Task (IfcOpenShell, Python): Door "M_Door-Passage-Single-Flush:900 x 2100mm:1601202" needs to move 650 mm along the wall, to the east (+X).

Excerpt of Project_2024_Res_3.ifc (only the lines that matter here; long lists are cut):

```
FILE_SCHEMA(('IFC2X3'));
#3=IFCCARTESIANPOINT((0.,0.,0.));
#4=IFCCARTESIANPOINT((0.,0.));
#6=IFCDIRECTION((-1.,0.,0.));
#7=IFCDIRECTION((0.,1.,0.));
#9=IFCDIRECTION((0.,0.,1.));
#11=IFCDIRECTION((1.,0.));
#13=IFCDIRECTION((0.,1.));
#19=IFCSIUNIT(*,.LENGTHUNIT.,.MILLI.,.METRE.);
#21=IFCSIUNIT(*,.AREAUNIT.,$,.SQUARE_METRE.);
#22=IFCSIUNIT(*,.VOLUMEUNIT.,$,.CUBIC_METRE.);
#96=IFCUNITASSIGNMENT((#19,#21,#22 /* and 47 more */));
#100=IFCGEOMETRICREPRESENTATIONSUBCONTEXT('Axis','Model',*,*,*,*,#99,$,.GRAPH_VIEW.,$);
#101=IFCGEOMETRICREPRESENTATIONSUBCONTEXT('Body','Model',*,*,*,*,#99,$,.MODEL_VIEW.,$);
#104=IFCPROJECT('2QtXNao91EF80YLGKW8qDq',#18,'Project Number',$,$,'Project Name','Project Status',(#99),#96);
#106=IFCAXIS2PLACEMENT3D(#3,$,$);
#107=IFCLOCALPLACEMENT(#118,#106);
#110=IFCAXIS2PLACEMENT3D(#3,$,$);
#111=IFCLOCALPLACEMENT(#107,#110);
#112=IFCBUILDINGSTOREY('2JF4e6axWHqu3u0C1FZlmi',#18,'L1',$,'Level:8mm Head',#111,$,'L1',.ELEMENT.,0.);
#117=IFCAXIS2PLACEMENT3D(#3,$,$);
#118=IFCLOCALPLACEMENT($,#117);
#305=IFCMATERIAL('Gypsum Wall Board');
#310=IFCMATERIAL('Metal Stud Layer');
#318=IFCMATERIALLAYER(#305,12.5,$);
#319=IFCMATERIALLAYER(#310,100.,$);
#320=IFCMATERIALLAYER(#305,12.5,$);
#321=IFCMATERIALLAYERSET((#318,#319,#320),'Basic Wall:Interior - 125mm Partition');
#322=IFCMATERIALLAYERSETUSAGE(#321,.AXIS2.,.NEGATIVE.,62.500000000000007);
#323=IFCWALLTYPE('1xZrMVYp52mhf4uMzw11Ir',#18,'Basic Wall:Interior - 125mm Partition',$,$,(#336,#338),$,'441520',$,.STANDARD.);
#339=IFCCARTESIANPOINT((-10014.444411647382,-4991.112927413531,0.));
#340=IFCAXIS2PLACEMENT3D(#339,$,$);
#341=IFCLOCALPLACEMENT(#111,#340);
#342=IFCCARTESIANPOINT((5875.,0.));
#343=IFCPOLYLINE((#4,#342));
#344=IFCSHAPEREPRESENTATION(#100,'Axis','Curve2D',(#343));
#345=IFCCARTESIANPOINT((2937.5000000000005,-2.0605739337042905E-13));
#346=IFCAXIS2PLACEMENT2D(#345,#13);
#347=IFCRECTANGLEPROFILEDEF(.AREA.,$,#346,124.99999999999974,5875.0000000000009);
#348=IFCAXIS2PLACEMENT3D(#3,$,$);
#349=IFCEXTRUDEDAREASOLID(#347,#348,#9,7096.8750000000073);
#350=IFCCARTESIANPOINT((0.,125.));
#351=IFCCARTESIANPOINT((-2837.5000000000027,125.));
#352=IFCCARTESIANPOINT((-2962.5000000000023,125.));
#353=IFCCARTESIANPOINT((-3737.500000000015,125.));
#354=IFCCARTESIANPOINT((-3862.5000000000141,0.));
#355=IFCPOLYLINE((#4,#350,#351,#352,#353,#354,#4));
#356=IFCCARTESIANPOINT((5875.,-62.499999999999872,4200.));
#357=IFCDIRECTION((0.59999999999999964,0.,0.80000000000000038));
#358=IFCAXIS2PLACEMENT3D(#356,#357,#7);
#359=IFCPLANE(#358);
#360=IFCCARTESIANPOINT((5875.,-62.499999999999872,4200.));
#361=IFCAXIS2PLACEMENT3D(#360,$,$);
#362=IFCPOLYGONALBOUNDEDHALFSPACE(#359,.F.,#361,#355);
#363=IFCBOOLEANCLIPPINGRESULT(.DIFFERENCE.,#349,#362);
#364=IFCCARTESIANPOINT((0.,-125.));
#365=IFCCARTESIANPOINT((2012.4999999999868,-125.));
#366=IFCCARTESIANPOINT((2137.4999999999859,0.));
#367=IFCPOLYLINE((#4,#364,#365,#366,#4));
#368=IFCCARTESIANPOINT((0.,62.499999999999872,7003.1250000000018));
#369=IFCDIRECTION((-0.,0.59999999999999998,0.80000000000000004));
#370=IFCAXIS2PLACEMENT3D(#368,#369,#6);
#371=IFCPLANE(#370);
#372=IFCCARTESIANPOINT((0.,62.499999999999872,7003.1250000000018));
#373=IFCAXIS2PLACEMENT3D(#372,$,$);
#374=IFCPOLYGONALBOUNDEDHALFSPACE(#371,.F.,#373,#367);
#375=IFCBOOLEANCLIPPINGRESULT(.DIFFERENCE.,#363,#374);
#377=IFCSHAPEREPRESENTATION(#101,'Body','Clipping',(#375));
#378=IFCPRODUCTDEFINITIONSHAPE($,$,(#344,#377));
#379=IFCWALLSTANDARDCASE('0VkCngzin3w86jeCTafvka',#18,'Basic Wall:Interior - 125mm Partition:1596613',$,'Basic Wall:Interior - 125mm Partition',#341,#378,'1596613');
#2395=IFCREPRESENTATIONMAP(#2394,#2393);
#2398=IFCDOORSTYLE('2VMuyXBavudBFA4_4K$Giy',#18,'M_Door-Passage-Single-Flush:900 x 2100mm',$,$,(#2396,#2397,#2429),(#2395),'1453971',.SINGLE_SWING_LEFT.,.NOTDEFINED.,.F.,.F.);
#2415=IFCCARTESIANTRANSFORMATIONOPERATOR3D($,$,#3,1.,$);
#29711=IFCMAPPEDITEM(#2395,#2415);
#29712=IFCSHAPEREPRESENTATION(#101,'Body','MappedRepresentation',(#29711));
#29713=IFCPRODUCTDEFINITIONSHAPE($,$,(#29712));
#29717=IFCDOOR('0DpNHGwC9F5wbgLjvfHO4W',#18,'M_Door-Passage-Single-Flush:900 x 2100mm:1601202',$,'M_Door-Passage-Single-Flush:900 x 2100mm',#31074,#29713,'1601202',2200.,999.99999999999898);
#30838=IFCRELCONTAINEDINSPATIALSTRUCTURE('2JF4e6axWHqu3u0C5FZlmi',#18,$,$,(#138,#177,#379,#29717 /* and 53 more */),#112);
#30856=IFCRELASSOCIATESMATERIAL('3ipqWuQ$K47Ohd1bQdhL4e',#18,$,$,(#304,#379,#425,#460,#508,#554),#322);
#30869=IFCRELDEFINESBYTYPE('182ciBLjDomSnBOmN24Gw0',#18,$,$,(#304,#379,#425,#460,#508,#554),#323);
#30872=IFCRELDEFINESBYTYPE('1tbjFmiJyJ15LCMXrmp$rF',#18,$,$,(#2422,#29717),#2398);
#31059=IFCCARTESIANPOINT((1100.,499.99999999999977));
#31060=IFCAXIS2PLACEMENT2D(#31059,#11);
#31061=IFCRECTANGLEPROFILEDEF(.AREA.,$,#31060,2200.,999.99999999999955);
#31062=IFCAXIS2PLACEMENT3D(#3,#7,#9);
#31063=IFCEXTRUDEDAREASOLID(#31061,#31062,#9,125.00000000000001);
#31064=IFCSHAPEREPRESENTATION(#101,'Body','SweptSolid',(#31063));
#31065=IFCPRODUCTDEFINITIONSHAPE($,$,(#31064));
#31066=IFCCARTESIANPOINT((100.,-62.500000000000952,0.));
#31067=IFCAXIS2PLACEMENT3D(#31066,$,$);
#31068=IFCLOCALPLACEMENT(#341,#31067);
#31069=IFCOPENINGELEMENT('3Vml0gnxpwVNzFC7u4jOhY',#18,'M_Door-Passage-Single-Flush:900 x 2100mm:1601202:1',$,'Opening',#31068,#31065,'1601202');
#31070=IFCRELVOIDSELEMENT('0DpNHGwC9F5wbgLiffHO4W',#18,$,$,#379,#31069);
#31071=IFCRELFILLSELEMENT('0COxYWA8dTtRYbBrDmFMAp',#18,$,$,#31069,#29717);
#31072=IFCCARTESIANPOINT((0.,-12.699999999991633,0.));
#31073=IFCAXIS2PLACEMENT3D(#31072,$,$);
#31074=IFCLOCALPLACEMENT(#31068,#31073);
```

```python
import ifcopenshell
import ifcopenshell.api.geometry
import ifcopenshell.util.placement

model = ifcopenshell.open("Project_2024_Res_3.ifc")

door = model.by_guid("0DpNHGwC9F5wbgLjvfHO4W")
opening = door.FillsVoids[0].RelatingOpeningElement
wall = opening.VoidsElements[0].RelatingBuildingElement

wall_matrix = ifcopenshell.util.placement.get_local_placement(wall.ObjectPlacement)
shift = wall_matrix[:3, 0] * 650.0
before = ifcopenshell.util.placement.get_local_placement(door.ObjectPlacement)[:3, 3].copy()

# The door is placed relative to its opening, so it follows when the opening moves.
matrix = ifcopenshell.util.placement.get_local_placement(opening.ObjectPlacement)
matrix[:3, 3] += shift
ifcopenshell.api.geometry.edit_object_placement(
    model, product=opening, matrix=matrix, is_si=False, should_transform_children=True
)

after = ifcopenshell.util.placement.get_local_placement(door.ObjectPlacement)[:3, 3]
print("door moved by", (after - before).round(3) + 0.0)

model.write("Project_2024_Res_3_rev.ifc")
```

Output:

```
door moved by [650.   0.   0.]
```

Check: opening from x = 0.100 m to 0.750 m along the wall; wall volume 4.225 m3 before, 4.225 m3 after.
